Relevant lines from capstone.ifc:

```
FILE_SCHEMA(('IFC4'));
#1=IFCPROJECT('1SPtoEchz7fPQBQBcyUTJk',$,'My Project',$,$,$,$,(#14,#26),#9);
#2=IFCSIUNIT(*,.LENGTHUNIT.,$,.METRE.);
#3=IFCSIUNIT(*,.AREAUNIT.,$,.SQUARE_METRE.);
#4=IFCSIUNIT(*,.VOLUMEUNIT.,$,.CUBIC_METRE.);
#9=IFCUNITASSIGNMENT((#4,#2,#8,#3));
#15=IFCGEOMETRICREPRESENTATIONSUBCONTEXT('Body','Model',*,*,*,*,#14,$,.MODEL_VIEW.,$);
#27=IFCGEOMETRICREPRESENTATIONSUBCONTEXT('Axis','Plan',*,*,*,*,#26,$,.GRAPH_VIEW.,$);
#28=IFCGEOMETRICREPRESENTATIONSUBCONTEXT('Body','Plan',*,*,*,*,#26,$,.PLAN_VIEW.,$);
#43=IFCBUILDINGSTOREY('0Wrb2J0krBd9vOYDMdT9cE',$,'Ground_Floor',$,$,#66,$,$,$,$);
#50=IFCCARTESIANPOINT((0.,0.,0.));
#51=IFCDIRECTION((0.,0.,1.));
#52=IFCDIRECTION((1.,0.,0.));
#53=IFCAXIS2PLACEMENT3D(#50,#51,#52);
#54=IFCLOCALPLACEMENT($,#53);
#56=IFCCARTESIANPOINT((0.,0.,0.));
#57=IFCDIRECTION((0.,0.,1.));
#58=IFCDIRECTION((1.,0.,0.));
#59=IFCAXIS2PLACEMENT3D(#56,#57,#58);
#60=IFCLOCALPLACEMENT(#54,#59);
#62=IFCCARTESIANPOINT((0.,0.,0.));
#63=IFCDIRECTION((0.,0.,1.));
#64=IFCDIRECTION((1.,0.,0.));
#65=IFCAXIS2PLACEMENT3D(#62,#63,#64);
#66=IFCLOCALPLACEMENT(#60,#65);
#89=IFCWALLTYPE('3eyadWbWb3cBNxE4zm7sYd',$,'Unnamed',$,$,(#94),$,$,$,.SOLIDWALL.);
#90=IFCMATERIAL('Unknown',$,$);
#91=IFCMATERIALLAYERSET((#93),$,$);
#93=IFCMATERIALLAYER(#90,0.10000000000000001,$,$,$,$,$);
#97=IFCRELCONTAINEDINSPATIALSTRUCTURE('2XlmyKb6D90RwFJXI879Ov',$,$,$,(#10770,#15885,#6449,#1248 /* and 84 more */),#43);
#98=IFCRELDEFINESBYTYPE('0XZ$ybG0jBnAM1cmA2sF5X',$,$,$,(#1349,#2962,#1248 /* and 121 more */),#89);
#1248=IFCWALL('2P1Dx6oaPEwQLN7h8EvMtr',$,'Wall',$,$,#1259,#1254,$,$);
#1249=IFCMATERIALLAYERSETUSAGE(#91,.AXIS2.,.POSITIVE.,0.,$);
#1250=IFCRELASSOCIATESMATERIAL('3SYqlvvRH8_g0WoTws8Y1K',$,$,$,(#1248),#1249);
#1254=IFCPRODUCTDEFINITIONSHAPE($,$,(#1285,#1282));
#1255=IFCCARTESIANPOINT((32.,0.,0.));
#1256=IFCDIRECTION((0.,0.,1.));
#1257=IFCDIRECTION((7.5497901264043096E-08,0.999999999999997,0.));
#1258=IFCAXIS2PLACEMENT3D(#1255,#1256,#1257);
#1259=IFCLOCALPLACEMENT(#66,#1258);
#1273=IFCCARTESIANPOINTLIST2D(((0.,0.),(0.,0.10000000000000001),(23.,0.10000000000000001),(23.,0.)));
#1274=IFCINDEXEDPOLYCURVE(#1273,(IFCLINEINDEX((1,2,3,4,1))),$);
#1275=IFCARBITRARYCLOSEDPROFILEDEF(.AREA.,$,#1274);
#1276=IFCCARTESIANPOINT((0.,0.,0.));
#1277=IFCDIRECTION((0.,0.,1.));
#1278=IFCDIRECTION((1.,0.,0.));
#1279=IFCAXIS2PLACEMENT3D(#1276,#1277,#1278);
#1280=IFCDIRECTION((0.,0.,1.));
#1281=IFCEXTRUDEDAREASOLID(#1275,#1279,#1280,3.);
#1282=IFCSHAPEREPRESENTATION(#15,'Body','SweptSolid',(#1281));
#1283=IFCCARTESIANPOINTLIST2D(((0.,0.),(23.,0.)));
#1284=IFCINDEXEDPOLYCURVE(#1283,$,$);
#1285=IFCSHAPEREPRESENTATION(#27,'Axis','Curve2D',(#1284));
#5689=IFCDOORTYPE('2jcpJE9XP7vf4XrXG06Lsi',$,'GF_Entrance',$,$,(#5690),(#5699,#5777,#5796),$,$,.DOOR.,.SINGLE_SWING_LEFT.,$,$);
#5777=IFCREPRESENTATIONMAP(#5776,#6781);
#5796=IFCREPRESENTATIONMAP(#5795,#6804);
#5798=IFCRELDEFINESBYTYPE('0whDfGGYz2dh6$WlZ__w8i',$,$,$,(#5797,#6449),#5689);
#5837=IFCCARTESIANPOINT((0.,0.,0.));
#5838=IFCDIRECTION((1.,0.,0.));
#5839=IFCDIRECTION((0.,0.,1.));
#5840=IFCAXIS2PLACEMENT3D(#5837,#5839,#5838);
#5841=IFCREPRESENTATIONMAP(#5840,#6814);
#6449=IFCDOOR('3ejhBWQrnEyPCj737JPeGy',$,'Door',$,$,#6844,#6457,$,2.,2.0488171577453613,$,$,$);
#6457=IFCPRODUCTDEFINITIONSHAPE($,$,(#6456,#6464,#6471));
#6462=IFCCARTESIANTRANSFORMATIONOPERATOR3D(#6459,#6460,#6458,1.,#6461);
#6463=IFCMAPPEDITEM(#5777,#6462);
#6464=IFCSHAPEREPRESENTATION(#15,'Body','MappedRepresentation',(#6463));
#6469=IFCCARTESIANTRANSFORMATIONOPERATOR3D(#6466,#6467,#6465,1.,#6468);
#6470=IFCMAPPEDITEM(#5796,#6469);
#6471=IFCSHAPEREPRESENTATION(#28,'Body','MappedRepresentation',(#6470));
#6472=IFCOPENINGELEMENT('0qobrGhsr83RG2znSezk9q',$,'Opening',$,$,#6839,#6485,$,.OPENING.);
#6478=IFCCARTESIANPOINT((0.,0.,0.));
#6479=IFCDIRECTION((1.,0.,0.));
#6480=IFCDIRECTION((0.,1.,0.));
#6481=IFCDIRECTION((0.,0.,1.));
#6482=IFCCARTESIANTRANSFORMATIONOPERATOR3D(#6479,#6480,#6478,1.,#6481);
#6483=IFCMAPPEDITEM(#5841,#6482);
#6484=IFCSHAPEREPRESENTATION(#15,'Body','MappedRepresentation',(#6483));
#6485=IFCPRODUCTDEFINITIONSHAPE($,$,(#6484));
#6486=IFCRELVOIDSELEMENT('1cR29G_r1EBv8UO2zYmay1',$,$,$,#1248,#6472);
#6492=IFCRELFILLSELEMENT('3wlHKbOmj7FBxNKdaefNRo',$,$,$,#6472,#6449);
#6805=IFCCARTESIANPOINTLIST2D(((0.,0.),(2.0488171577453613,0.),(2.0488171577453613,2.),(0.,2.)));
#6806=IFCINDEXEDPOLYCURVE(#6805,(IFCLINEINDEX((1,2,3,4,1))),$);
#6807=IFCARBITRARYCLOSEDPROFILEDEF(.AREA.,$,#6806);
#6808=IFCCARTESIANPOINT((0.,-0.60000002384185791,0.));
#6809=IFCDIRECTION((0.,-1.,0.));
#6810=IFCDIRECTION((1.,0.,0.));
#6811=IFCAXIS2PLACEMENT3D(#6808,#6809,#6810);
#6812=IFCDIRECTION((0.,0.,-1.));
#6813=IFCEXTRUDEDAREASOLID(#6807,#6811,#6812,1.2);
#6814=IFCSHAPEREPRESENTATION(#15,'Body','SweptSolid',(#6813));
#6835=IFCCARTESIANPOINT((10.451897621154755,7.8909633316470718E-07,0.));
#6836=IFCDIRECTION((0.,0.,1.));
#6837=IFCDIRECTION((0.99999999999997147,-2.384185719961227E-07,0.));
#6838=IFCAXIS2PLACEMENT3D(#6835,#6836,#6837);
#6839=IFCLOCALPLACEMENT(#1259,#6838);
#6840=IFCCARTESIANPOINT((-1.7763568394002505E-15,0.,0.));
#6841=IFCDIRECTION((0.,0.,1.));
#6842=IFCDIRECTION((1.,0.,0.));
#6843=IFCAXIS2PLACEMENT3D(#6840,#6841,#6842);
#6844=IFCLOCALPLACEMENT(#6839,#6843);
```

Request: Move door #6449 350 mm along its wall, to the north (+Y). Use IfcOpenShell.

```python
import ifcopenshell
import ifcopenshell.api.geometry
import ifcopenshell.util.placement
import ifcopenshell.util.unit

model = ifcopenshell.open("capstone.ifc")
unit_scale = ifcopenshell.util.unit.calculate_unit_scale(model)

door = model.by_guid("3ejhBWQrnEyPCj737JPeGy")
opening = door.FillsVoids[0].RelatingOpeningElement
wall = opening.VoidsElements[0].RelatingBuildingElement

wall_matrix = ifcopenshell.util.placement.get_local_placement(wall.ObjectPlacement)
shift = wall_matrix[:3, 0] * 0.35 / unit_scale
before = ifcopenshell.util.placement.get_local_placement(door.ObjectPlacement)[:3, 3].copy()

# The door is placed relative to its opening, so it follows when the opening moves.
matrix = ifcopenshell.util.placement.get_local_placement(opening.ObjectPlacement)
matrix[:3, 3] += shift
ifcopenshell.api.geometry.edit_object_placement(
    model, product=opening, matrix=matrix, is_si=False, should_transform_children=True
)

after = ifcopenshell.util.placement.get_local_placement(door.ObjectPlacement)[:3, 3]
print("door moved by", (after - before).round(3) + 0.0)

model.write("capstone_rev.ifc")
```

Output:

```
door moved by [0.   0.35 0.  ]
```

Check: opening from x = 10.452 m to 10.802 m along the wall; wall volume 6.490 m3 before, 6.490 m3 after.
